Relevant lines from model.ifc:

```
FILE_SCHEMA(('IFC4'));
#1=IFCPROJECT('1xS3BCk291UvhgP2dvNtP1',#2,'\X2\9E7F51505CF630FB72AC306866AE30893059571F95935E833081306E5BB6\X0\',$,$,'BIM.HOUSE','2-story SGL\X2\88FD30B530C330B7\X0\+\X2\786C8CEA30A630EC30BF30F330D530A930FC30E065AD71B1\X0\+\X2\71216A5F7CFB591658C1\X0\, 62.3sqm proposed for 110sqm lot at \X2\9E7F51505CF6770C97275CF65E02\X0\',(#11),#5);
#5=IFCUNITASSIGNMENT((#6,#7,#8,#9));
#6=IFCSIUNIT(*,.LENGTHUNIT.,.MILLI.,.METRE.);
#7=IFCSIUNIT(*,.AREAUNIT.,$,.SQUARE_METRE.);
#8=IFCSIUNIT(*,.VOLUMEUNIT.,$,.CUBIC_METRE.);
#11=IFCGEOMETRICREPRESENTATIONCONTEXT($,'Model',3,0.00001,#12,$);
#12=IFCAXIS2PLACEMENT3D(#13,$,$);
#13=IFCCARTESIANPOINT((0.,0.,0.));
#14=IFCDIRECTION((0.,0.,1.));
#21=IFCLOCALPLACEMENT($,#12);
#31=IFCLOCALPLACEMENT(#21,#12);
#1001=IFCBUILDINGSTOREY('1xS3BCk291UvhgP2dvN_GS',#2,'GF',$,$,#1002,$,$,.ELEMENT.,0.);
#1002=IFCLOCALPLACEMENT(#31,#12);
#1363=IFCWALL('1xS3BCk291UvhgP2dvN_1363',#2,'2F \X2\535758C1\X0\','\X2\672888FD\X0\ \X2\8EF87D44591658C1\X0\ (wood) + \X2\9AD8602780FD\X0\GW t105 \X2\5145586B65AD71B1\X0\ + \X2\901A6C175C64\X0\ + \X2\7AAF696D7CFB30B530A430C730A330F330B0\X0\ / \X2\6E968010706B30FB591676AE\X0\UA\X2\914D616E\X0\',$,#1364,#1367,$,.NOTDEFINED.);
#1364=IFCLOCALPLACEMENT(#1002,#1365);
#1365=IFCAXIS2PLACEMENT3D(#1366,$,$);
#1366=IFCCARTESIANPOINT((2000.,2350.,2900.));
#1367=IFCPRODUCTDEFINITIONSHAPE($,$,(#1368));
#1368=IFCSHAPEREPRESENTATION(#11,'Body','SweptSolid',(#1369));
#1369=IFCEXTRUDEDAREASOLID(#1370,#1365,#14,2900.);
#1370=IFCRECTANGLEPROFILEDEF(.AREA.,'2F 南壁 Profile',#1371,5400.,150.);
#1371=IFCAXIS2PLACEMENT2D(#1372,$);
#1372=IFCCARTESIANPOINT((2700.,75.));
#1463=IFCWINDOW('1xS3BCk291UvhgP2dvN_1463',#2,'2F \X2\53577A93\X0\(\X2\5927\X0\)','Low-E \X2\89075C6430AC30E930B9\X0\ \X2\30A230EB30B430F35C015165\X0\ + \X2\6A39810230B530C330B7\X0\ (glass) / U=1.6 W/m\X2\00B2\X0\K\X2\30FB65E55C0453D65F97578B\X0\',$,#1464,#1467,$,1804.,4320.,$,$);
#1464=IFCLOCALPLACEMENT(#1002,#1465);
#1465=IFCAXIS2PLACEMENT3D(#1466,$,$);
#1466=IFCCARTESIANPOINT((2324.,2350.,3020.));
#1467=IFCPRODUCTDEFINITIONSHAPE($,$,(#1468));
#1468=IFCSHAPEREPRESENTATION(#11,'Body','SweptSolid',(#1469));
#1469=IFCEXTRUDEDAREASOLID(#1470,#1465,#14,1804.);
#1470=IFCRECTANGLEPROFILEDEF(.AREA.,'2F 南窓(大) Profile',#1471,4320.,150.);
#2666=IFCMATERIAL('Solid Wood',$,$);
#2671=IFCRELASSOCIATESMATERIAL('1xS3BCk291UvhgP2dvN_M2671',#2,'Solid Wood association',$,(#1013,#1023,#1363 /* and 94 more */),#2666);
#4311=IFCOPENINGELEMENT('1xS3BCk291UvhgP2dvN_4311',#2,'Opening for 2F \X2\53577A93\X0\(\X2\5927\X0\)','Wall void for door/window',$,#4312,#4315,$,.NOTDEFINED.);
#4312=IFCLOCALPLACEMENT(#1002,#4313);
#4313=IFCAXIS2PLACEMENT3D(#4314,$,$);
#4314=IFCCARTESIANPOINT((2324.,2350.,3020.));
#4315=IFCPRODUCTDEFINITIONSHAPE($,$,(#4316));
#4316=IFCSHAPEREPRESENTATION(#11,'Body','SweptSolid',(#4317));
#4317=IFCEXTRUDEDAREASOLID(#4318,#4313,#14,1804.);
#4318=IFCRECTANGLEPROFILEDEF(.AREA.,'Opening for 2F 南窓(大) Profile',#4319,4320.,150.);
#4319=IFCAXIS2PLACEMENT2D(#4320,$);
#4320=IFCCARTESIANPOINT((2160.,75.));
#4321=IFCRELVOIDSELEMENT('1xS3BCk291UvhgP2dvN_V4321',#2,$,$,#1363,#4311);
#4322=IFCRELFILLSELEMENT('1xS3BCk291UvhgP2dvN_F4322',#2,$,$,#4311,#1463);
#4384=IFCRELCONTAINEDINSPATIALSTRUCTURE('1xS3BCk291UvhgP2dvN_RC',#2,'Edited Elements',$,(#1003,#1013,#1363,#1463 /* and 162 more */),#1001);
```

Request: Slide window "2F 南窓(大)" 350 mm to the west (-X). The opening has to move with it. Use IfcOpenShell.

```python
import ifcopenshell
import ifcopenshell.api.geometry
import ifcopenshell.util.placement

model = ifcopenshell.open("model.ifc")

window = model.by_guid("1xS3BCk291UvhgP2dvN_1463")
opening = window.FillsVoids[0].RelatingOpeningElement
wall = opening.VoidsElements[0].RelatingBuildingElement

wall_matrix = ifcopenshell.util.placement.get_local_placement(wall.ObjectPlacement)
shift = wall_matrix[:3, 0] * -350.0
before = ifcopenshell.util.placement.get_local_placement(window.ObjectPlacement)[:3, 3].copy()

# The window is not placed relative to its opening, so move both.
for product in (opening, window):
    matrix = ifcopenshell.util.placement.get_local_placement(product.ObjectPlacement)
    matrix[:3, 3] += shift
    ifcopenshell.api.geometry.edit_object_placement(model, product=product, matrix=matrix, is_si=False)

after = ifcopenshell.util.placement.get_local_placement(window.ObjectPlacement)[:3, 3]
print("window moved by", (after - before).round(3) + 0.0)

model.write("model_updated.ifc")
```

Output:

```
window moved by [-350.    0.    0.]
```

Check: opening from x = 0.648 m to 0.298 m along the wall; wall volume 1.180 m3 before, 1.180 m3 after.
